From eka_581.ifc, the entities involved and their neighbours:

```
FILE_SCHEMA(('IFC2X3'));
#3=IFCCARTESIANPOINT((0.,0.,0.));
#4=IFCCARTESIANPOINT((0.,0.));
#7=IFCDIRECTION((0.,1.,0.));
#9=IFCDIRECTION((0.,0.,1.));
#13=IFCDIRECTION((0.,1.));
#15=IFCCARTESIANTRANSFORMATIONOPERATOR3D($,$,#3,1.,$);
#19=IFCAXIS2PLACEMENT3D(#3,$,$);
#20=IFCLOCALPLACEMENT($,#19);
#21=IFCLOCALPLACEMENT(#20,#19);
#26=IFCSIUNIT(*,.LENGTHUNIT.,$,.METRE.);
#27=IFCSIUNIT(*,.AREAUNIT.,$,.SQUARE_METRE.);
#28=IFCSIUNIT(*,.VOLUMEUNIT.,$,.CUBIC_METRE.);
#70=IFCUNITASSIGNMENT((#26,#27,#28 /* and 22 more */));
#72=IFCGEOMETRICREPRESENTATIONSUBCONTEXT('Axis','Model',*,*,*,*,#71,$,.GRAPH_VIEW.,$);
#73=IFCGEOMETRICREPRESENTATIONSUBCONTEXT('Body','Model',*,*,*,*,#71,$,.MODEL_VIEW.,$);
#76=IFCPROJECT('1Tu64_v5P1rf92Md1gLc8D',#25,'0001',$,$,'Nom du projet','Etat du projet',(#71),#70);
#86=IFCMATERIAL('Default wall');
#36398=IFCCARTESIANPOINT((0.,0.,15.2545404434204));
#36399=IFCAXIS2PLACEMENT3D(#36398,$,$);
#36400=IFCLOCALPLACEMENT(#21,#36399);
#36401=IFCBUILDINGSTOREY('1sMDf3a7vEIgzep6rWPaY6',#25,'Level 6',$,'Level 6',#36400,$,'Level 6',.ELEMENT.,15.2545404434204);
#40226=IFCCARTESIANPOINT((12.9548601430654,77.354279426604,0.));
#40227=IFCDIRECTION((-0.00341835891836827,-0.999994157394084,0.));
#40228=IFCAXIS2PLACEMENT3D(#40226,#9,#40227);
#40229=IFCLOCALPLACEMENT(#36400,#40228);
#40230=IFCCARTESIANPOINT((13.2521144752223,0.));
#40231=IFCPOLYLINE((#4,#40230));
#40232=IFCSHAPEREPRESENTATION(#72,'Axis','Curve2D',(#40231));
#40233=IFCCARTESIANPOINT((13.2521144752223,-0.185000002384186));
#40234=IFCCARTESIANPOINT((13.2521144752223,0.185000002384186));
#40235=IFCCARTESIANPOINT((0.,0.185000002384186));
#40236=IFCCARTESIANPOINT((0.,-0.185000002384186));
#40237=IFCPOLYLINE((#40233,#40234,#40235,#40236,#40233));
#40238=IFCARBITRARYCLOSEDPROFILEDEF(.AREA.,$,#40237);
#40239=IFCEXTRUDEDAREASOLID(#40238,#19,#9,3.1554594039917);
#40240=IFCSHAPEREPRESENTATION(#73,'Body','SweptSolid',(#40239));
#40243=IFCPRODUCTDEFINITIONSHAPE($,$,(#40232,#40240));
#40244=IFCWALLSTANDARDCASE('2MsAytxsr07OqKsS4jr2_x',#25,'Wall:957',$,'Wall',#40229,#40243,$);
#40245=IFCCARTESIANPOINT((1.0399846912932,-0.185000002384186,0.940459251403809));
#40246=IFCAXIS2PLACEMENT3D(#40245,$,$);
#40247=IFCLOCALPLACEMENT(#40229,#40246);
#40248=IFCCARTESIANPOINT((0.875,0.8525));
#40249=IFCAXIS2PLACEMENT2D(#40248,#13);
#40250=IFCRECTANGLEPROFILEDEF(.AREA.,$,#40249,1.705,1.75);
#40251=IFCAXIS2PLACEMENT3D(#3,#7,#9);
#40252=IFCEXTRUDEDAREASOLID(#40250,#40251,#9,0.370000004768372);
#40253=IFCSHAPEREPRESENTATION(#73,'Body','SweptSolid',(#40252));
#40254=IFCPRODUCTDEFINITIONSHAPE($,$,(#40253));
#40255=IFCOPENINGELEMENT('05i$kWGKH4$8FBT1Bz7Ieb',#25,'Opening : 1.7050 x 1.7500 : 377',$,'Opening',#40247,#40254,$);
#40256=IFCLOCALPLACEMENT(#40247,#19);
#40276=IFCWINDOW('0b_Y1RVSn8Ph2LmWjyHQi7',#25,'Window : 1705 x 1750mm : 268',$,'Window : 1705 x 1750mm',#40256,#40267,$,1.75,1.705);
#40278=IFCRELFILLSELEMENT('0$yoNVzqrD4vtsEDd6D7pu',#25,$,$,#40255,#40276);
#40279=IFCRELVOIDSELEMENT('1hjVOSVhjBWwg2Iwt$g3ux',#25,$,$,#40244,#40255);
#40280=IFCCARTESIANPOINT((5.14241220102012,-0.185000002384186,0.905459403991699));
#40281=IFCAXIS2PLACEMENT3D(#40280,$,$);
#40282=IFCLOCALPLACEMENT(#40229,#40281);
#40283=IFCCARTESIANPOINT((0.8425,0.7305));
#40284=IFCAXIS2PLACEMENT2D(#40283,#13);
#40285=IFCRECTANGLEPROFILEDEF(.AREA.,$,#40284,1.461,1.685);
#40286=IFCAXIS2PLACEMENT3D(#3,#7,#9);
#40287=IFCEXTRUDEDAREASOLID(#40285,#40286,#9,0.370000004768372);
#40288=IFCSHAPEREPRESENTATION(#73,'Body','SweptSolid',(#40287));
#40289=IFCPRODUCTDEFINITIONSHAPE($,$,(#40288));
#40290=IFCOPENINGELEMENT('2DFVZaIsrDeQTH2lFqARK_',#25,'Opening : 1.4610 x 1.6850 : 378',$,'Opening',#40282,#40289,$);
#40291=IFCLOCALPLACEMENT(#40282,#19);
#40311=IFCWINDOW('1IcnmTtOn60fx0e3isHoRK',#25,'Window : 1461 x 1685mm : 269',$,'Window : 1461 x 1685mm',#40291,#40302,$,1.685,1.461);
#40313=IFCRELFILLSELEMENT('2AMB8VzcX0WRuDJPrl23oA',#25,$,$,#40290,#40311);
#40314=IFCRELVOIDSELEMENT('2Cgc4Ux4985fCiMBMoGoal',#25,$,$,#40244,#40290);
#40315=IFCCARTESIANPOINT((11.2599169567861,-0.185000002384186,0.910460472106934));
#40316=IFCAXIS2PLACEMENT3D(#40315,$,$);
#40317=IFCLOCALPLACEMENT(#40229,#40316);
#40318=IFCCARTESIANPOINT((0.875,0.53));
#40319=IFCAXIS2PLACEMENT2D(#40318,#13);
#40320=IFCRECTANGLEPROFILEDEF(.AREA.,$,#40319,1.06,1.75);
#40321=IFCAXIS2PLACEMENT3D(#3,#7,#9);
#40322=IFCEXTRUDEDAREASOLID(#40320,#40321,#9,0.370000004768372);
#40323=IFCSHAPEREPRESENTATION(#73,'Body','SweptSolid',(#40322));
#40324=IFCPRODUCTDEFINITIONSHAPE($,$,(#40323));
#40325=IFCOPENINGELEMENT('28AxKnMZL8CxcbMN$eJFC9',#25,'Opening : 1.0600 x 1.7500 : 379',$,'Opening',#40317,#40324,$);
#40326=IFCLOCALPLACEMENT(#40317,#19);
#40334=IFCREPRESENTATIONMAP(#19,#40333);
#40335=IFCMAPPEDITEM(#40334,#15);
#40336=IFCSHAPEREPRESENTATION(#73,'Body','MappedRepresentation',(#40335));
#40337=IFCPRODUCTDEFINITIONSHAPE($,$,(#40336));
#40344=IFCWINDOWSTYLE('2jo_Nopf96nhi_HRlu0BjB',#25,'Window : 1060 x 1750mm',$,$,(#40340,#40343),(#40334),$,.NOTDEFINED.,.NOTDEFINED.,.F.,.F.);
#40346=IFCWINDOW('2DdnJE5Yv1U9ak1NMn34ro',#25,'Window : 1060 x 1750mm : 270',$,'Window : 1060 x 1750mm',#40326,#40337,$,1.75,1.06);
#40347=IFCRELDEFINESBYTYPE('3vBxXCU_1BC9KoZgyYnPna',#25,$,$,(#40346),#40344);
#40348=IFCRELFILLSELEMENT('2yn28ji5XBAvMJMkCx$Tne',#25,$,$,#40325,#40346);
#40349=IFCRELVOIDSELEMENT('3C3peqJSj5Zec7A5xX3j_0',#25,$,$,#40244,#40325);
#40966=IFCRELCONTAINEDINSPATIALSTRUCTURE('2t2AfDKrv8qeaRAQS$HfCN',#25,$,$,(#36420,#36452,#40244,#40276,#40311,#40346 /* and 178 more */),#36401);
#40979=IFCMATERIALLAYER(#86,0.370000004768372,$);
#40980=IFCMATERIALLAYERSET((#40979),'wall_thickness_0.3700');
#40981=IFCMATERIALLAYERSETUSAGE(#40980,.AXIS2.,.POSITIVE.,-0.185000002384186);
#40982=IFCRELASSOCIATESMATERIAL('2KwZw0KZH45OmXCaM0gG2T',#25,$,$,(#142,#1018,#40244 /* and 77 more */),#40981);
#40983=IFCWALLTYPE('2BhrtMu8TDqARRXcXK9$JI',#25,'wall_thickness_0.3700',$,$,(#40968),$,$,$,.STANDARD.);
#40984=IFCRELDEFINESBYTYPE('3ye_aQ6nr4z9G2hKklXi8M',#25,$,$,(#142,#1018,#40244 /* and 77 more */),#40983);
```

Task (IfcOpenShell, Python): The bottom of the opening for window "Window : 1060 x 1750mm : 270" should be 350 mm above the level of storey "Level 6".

```python
import numpy as np
import ifcopenshell
import ifcopenshell.api.geometry
import ifcopenshell.geom
import ifcopenshell.util.element
import ifcopenshell.util.placement
import ifcopenshell.util.shape
import ifcopenshell.util.unit

model = ifcopenshell.open("eka_581.ifc")
unit_scale = ifcopenshell.util.unit.calculate_unit_scale(model)

window = model.by_id(40346)
opening = window.FillsVoids[0].RelatingOpeningElement
storey = ifcopenshell.util.element.get_container(window, ifc_class="IfcBuildingStorey")
level = ifcopenshell.util.placement.get_local_placement(storey.ObjectPlacement)[2, 3]

# The opening's origin need not be at the sill, so measure its lowest point.
shape = ifcopenshell.geom.create_shape(ifcopenshell.geom.settings(), opening)
bottom = ifcopenshell.util.shape.get_shape_bottom_elevation(shape, shape.geometry) / unit_scale
dz = level + 0.35 / unit_scale - bottom

shift = np.array([0.0, 0.0, dz])
# The window is placed relative to its opening, so it follows when the opening moves.
matrix = ifcopenshell.util.placement.get_local_placement(opening.ObjectPlacement)
matrix[:3, 3] += shift
ifcopenshell.api.geometry.edit_object_placement(
    model, product=opening, matrix=matrix, is_si=False, should_transform_children=True
)

print(f"moved by {dz * unit_scale:+.3f} m")

model.write("eka_581_v2.ifc")
```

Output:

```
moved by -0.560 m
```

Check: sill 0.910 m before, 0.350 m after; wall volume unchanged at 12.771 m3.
